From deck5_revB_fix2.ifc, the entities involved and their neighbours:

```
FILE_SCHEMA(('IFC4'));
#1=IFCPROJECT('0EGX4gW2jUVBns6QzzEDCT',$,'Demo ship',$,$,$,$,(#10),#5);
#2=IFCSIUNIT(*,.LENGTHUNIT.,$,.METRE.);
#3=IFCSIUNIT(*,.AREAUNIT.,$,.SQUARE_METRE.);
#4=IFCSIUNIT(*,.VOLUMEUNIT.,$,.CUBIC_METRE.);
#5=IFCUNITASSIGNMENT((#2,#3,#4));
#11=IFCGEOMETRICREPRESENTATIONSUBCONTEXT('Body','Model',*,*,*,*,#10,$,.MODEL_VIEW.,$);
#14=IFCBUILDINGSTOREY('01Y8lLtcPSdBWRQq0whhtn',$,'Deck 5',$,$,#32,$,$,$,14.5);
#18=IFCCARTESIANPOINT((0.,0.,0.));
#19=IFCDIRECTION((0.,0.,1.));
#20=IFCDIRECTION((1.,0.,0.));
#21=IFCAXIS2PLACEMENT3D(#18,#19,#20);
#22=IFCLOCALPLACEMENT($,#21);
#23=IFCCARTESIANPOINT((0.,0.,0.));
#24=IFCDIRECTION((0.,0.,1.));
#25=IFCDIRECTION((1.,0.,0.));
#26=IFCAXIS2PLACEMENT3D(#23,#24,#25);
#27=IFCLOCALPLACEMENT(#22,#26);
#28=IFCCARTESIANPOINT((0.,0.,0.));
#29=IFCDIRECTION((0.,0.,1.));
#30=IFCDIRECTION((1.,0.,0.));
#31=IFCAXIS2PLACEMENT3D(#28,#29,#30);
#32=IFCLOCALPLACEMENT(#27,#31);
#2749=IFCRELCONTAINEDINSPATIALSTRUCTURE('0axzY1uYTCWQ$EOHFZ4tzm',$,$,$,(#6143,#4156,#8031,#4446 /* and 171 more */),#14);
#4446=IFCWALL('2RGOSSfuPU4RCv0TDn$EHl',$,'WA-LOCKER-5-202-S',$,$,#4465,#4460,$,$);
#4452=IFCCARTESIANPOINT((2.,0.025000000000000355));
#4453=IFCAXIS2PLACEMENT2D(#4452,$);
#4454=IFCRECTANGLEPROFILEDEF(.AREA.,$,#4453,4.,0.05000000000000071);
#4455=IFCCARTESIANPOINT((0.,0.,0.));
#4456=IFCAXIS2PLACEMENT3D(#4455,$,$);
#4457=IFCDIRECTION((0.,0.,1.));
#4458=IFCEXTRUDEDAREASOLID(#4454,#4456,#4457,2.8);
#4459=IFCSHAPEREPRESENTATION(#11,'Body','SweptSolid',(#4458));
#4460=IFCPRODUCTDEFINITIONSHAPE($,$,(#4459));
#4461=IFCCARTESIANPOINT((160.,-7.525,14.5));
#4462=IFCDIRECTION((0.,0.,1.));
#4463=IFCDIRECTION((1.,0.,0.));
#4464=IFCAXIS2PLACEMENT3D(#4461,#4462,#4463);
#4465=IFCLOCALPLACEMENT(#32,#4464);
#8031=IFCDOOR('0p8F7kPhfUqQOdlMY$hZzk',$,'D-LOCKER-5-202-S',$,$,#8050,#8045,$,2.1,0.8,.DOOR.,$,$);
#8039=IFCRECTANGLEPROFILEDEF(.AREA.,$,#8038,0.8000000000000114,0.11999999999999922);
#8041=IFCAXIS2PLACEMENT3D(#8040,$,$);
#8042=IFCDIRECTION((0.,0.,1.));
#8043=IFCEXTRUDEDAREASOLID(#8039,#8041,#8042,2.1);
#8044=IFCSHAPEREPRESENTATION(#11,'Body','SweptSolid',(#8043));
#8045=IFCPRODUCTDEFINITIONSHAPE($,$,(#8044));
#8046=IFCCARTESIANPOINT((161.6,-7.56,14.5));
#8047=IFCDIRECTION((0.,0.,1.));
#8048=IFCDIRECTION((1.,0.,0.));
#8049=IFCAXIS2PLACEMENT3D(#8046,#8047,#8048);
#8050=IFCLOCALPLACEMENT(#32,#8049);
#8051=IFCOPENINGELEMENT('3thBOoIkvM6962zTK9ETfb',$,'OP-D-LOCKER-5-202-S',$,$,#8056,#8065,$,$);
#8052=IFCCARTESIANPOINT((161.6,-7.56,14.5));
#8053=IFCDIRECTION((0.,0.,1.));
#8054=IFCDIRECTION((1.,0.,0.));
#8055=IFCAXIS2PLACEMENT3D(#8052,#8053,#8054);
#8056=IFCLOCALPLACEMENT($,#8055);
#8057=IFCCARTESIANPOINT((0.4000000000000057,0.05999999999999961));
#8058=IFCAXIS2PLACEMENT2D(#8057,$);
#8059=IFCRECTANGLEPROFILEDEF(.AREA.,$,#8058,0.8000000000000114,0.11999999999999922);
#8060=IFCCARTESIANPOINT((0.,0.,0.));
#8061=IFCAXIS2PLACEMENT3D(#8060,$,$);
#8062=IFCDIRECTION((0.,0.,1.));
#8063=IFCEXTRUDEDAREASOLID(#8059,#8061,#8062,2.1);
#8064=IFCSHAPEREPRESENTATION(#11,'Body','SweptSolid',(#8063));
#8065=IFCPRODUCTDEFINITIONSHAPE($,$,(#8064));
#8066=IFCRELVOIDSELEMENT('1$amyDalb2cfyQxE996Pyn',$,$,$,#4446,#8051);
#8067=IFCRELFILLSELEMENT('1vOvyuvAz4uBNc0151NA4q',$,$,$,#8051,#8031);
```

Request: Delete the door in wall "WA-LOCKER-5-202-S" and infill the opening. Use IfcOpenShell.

```python
import ifcopenshell
import ifcopenshell.api.feature
import ifcopenshell.api.root
import ifcopenshell.geom
import ifcopenshell.util.shape

model = ifcopenshell.open("deck5_revB_fix2.ifc")
settings = ifcopenshell.geom.settings()


def volume(element):
    """Net volume in cubic metres, openings subtracted."""
    shape = ifcopenshell.geom.create_shape(settings, element)
    return ifcopenshell.util.shape.get_volume(shape.geometry)


door = model.by_guid("0p8F7kPhfUqQOdlMY$hZzk")
opening = door.FillsVoids[0].RelatingOpeningElement
wall = opening.VoidsElements[0].RelatingBuildingElement
before = volume(wall)

ifcopenshell.api.root.remove_product(model, product=door)
ifcopenshell.api.feature.remove_feature(model, feature=opening)

after = volume(wall)

print(f"wall volume {before:.3f} -> {after:.3f} m3")

model.write("deck5_revB_fix2_updated.ifc")
```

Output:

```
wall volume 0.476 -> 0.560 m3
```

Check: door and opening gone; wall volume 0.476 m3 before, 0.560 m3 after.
